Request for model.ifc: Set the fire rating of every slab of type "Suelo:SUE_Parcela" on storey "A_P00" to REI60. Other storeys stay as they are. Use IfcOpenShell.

First a look at what the model holds.

```python
import ifcopenshell
import ifcopenshell.util.element

model = ifcopenshell.open("model.ifc")
print(model.schema)
storey = next(s for s in model.by_type("IfcBuildingStorey") if s.Name == "A_P00")
slabs = [e for e in ifcopenshell.util.element.get_decomposition(storey) if e.is_a("IfcSlab")]
seen = {}
for e in slabs:
    element_type = ifcopenshell.util.element.get_type(e)
    key = (element_type.Name if element_type != e and element_type else None, ifcopenshell.util.element.get_pset(e, "Pset_SlabCommon", "FireRating"))
    seen[key] = seen.get(key, 0) + 1
for (name, value), count in sorted(seen.items(), key=str):
    print(count, "x", name, "|", value)
```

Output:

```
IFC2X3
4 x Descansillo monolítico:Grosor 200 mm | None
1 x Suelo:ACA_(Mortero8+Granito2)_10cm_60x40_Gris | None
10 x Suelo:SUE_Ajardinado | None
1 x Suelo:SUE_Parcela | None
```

```python
import ifcopenshell
import ifcopenshell.api.pset
import ifcopenshell.util.element

model = ifcopenshell.open("model.ifc")

storey = next(s for s in model.by_type("IfcBuildingStorey") if s.Name == "A_P00")
slabs = [e for e in ifcopenshell.util.element.get_decomposition(storey) if e.is_a("IfcSlab")]

count = 0
for e in slabs:
    element_type = ifcopenshell.util.element.get_type(e)
    if element_type in (None, e) or element_type.Name != "Suelo:SUE_Parcela":
        continue
    # add_pset returns the element's existing set when there is one.
    pset = ifcopenshell.api.pset.add_pset(model, product=e, name="Pset_SlabCommon")
    ifcopenshell.api.pset.edit_pset(model, pset=pset, properties={"FireRating": "REI60"})
    count += 1

print(count, "slabs updated")

model.write("model_rev.ifc")
```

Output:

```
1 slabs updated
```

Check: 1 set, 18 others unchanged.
